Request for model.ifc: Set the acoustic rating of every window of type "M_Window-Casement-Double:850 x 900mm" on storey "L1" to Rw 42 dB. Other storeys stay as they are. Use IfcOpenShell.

First a look at what the model holds.

```python
import ifcopenshell
import ifcopenshell.util.element

model = ifcopenshell.open("model.ifc")
print(model.schema)
storey = next(s for s in model.by_type("IfcBuildingStorey") if s.Name == "L1")
windows = [e for e in ifcopenshell.util.element.get_decomposition(storey) if e.is_a("IfcWindow")]
seen = {}
for e in windows:
    element_type = ifcopenshell.util.element.get_type(e)
    key = (element_type.Name if element_type != e and element_type else None, ifcopenshell.util.element.get_pset(e, "Pset_WindowCommon", "AcousticRating"))
    seen[key] = seen.get(key, 0) + 1
for (name, value), count in sorted(seen.items(), key=str):
    print(count, "x", name, "|", value)
```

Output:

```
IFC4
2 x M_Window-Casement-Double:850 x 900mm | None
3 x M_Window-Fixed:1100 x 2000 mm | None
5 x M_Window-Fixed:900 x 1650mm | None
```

```python
import ifcopenshell
import ifcopenshell.api.pset
import ifcopenshell.util.element

model = ifcopenshell.open("model.ifc")

storey = next(s for s in model.by_type("IfcBuildingStorey") if s.Name == "L1")
windows = [e for e in ifcopenshell.util.element.get_decomposition(storey) if e.is_a("IfcWindow")]

count = 0
for e in windows:
    element_type = ifcopenshell.util.element.get_type(e)
    if element_type in (None, e) or element_type.Name != "M_Window-Casement-Double:850 x 900mm":
        continue
    # add_pset returns the element's existing set when there is one.
    pset = ifcopenshell.api.pset.add_pset(model, product=e, name="Pset_WindowCommon")
    ifcopenshell.api.pset.edit_pset(model, pset=pset, properties={"AcousticRating": "Rw 42 dB"})
    count += 1

print(count, "windows updated")

model.write("model_rev.ifc")
```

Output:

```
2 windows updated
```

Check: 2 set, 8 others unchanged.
